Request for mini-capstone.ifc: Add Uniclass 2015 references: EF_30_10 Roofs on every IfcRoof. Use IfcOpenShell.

First a look at what the model holds.

```python
import ifcopenshell

model = ifcopenshell.open("mini-capstone.ifc")
print(model.schema)
print("classifications:", [c.Name for c in model.by_type("IfcClassification")])
for ifc_class in ("IfcDoor", "IfcRoof", "IfcStair", "IfcWall", "IfcWindow"):
    print(ifc_class, len(model.by_type(ifc_class)))
```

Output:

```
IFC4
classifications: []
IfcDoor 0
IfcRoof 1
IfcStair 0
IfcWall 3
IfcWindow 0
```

```python
import ifcopenshell
import ifcopenshell.api.classification

model = ifcopenshell.open("mini-capstone.ifc")

system = ifcopenshell.api.classification.add_classification(model, classification="Uniclass 2015")

codes = {
    "IfcRoof": ("EF_30_10", "Roofs"),
}
for ifc_class, (code, name) in codes.items():
    products = model.by_type(ifc_class)
    ifcopenshell.api.classification.add_reference(
        model, products=products, classification=system, identification=code, name=name
    )
    print(code, len(products))

model.write("mini-capstone_updated.ifc")
```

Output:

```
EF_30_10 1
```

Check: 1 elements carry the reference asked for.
